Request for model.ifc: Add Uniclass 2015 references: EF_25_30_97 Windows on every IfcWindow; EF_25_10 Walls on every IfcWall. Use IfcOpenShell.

First a look at what the model holds.

```python
import ifcopenshell

model = ifcopenshell.open("model.ifc")
print(model.schema)
print("classifications:", [c.Name for c in model.by_type("IfcClassification")])
for ifc_class in ("IfcDoor", "IfcRoof", "IfcStair", "IfcWall", "IfcWindow"):
    print(ifc_class, len(model.by_type(ifc_class)))
```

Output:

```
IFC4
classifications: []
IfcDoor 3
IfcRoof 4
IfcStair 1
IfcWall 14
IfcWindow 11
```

```python
import ifcopenshell
import ifcopenshell.api.classification

model = ifcopenshell.open("model.ifc")

system = ifcopenshell.api.classification.add_classification(model, classification="Uniclass 2015")

codes = {
    "IfcWindow": ("EF_25_30_97", "Windows"),
    "IfcWall": ("EF_25_10", "Walls"),
}
for ifc_class, (code, name) in codes.items():
    products = model.by_type(ifc_class)
    ifcopenshell.api.classification.add_reference(
        model, products=products, classification=system, identification=code, name=name
    )
    print(code, len(products))

model.write("model_v2.ifc")
```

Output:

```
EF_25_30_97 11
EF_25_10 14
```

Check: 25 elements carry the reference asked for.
